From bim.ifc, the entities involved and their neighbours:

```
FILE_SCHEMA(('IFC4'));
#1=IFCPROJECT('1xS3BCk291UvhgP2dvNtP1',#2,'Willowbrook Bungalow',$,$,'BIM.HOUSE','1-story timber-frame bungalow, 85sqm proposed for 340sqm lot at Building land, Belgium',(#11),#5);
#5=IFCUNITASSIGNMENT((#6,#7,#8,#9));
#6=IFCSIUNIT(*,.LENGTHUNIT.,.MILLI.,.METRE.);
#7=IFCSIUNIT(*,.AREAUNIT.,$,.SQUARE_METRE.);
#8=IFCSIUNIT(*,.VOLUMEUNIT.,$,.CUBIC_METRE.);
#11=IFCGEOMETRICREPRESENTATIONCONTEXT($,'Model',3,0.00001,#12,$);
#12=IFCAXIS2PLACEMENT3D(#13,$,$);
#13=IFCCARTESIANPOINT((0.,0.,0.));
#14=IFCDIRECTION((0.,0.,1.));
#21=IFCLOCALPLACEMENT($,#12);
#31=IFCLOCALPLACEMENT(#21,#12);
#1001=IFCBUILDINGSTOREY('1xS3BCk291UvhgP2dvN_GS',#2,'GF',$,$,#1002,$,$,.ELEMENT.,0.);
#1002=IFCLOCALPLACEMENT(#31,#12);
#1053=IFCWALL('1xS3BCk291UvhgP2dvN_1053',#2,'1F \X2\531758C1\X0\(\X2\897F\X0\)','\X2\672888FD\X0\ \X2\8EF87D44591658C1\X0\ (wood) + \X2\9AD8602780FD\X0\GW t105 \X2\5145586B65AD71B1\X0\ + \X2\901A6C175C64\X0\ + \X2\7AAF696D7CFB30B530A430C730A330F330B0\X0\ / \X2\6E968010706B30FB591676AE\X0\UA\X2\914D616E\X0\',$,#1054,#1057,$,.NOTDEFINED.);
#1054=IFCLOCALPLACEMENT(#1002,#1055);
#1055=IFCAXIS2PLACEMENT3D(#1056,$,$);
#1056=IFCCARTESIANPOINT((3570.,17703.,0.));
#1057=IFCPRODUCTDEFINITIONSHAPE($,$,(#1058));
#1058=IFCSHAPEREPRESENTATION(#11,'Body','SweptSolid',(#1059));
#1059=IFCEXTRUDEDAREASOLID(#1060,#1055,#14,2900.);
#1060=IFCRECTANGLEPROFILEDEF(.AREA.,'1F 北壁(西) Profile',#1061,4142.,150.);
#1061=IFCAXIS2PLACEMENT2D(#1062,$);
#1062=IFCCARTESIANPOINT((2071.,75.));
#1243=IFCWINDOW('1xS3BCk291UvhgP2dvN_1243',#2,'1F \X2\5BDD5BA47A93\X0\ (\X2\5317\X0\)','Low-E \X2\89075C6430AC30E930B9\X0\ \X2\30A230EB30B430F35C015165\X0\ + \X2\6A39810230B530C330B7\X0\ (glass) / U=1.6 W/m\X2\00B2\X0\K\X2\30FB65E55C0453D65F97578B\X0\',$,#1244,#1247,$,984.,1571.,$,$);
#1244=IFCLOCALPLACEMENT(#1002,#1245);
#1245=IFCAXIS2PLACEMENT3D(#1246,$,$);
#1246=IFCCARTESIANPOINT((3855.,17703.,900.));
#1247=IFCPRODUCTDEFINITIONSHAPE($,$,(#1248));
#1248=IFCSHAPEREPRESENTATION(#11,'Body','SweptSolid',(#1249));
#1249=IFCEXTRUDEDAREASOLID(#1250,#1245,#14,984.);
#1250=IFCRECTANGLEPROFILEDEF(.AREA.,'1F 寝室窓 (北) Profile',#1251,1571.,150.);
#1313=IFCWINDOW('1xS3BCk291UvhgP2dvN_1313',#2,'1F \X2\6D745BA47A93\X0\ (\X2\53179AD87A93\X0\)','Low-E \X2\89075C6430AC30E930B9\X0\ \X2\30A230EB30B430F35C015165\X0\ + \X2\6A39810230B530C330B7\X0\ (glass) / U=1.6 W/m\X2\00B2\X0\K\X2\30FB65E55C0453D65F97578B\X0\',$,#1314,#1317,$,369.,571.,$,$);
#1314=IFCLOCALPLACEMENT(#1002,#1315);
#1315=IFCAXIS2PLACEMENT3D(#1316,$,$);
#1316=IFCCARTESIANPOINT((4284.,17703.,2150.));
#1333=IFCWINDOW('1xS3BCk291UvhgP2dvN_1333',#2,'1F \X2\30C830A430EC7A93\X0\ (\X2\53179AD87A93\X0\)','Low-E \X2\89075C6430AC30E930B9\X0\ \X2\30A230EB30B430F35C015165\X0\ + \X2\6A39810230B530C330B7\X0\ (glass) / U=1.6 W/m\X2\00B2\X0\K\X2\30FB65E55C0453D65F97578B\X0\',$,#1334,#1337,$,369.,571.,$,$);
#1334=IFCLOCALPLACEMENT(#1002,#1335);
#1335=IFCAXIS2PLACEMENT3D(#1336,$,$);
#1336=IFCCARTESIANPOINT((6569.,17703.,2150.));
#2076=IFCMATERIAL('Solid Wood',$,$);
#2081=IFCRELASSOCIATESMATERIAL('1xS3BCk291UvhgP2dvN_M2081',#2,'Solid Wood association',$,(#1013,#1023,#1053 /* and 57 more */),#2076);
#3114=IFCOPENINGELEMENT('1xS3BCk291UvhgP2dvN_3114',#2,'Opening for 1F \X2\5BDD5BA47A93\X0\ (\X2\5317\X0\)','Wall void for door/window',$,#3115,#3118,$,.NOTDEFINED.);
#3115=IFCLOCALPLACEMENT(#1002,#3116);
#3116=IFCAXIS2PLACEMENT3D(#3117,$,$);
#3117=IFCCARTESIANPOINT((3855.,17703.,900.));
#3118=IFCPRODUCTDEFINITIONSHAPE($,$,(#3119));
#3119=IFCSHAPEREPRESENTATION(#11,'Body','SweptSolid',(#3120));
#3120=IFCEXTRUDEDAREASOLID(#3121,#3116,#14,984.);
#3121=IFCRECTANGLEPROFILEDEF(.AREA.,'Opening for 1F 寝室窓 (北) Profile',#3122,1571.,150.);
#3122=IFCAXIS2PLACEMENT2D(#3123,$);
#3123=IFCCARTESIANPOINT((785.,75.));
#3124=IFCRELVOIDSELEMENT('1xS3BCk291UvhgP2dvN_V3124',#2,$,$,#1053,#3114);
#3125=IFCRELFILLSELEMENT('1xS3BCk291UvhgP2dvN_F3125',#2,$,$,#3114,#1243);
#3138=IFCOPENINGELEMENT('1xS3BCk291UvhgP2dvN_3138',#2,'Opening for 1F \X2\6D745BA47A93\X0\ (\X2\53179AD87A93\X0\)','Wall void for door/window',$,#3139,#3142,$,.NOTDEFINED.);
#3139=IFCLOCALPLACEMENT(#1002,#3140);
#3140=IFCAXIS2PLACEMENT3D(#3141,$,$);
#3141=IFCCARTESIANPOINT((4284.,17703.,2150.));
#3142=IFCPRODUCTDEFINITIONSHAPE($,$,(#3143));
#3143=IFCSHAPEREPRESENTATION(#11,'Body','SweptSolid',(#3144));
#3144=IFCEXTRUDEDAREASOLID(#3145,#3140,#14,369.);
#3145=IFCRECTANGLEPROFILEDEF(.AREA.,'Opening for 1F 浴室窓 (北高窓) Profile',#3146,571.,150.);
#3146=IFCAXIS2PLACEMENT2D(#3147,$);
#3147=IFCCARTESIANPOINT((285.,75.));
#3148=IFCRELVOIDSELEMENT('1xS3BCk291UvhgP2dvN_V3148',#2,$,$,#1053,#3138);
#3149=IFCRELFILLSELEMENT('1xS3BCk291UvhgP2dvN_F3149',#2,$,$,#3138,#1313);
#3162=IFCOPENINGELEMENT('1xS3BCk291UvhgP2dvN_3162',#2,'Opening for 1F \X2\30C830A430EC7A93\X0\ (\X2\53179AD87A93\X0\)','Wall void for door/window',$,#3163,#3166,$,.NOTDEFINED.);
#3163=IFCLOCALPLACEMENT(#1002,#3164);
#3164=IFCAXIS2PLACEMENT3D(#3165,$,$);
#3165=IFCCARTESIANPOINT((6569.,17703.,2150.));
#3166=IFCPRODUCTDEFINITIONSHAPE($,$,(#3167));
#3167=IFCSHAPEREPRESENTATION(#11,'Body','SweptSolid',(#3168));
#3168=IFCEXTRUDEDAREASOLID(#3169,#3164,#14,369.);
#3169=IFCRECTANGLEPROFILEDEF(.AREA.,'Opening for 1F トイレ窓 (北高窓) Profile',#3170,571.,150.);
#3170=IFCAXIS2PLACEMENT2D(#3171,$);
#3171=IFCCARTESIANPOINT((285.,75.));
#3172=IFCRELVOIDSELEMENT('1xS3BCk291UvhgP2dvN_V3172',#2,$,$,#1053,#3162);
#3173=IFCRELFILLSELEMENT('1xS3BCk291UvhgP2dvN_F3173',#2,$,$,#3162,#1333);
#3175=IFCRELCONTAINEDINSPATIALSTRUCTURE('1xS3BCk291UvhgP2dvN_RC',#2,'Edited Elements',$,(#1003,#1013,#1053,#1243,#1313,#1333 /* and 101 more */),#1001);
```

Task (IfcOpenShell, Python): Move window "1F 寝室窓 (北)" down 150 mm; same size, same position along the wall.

```python
import numpy as np
import ifcopenshell
import ifcopenshell.api.geometry
import ifcopenshell.util.placement
import ifcopenshell.util.unit

model = ifcopenshell.open("bim.ifc")
unit_scale = ifcopenshell.util.unit.calculate_unit_scale(model)

window = model.by_id(1243)
opening = window.FillsVoids[0].RelatingOpeningElement
dz = -150.0

shift = np.array([0.0, 0.0, dz])
# The window is not placed relative to its opening, so move both.
for product in (opening, window):
    matrix = ifcopenshell.util.placement.get_local_placement(product.ObjectPlacement)
    matrix[:3, 3] += shift
    ifcopenshell.api.geometry.edit_object_placement(model, product=product, matrix=matrix, is_si=False)

print(f"moved by {dz * unit_scale:+.3f} m")

model.write("bim-out.ifc")
```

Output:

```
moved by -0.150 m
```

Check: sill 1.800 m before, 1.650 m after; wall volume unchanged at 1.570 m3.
